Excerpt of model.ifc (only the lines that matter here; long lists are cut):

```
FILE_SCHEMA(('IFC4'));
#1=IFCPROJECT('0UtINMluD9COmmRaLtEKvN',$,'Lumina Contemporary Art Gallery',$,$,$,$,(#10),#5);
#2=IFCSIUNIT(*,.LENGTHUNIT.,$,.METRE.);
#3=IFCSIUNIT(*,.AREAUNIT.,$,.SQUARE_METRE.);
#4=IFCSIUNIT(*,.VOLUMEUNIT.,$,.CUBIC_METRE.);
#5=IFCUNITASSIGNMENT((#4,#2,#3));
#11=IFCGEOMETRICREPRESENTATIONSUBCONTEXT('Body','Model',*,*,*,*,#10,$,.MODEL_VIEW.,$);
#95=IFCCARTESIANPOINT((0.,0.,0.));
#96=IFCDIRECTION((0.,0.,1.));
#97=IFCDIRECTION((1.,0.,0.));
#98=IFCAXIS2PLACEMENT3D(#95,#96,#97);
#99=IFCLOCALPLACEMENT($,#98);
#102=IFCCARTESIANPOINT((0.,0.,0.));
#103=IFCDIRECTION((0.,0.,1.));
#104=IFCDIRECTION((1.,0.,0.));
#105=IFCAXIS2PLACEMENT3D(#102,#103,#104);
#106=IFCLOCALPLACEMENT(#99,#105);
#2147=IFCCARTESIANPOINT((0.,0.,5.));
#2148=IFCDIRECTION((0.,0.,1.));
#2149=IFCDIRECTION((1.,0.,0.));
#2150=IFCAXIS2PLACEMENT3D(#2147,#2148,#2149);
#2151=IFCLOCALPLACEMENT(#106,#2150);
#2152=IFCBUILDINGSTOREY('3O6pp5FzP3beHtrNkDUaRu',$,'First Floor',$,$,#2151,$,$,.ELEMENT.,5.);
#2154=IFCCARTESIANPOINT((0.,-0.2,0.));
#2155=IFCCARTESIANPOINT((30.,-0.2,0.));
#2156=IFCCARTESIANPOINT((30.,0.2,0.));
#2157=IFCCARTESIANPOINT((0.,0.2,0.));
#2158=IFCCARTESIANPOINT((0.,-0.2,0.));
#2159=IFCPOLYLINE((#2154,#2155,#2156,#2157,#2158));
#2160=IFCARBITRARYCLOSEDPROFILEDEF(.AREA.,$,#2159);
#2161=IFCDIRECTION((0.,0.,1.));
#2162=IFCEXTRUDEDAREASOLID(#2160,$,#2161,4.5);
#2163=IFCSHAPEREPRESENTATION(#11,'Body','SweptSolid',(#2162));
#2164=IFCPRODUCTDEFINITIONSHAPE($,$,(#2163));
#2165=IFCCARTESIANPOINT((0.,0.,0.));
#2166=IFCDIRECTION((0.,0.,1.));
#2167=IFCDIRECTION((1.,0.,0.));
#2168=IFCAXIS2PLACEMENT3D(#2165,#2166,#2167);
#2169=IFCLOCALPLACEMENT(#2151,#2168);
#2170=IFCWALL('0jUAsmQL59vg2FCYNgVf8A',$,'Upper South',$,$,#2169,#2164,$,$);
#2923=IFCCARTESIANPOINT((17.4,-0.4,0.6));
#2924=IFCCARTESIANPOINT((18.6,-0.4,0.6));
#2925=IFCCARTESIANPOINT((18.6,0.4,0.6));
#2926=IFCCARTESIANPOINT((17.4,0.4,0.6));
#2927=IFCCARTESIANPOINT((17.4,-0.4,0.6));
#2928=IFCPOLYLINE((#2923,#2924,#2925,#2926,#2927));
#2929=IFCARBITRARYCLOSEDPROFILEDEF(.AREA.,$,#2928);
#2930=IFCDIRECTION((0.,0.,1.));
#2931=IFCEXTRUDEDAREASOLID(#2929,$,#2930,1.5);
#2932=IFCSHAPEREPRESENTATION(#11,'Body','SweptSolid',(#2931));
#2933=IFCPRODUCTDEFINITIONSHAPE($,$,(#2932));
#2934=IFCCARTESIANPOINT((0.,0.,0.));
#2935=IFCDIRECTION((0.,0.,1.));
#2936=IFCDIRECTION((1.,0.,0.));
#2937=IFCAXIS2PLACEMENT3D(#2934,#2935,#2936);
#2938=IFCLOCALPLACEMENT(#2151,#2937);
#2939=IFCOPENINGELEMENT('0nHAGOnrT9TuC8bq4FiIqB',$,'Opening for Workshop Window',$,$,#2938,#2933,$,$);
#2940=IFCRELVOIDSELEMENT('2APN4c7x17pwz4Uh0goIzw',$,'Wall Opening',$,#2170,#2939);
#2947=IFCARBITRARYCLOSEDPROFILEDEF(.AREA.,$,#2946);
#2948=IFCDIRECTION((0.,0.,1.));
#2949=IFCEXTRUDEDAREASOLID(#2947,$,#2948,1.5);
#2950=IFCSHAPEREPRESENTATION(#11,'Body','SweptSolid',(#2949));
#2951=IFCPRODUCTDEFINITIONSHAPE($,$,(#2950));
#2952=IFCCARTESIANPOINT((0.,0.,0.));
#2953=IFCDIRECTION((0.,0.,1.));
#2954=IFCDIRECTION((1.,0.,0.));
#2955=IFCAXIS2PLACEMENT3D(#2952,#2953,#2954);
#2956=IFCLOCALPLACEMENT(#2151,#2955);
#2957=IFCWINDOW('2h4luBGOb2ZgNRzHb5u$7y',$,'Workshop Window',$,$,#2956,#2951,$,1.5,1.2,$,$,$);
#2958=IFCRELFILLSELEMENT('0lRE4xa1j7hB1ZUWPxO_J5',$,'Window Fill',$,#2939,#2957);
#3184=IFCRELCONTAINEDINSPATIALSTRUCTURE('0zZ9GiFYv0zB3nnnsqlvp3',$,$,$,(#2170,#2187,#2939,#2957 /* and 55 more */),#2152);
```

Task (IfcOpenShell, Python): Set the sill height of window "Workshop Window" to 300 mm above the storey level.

```python
import numpy as np
import ifcopenshell
import ifcopenshell.api.geometry
import ifcopenshell.geom
import ifcopenshell.util.element
import ifcopenshell.util.placement
import ifcopenshell.util.shape
import ifcopenshell.util.unit

model = ifcopenshell.open("model.ifc")
unit_scale = ifcopenshell.util.unit.calculate_unit_scale(model)

window = model.by_id(2957)
opening = window.FillsVoids[0].RelatingOpeningElement
storey = ifcopenshell.util.element.get_container(window, ifc_class="IfcBuildingStorey")
level = ifcopenshell.util.placement.get_local_placement(storey.ObjectPlacement)[2, 3]

# The opening's origin need not be at the sill, so measure its lowest point.
shape = ifcopenshell.geom.create_shape(ifcopenshell.geom.settings(), opening)
bottom = ifcopenshell.util.shape.get_shape_bottom_elevation(shape, shape.geometry) / unit_scale
dz = level + 0.3 - bottom

shift = np.array([0.0, 0.0, dz])
# The window is not placed relative to its opening, so move both.
for product in (opening, window):
    matrix = ifcopenshell.util.placement.get_local_placement(product.ObjectPlacement)
    matrix[:3, 3] += shift
    ifcopenshell.api.geometry.edit_object_placement(model, product=product, matrix=matrix, is_si=False)

print(f"moved by {dz * unit_scale:+.3f} m")

model.write("model_updated.ifc")
```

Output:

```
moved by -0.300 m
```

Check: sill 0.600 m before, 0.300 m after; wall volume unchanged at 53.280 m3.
